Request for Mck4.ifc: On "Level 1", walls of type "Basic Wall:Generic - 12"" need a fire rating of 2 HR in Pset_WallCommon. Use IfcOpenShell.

First a look at what the model holds.

```python
import ifcopenshell
import ifcopenshell.util.element

model = ifcopenshell.open("Mck4.ifc")
print(model.schema)
storey = next(s for s in model.by_type("IfcBuildingStorey") if s.Name == "Level 1")
walls = [e for e in ifcopenshell.util.element.get_decomposition(storey) if e.is_a("IfcWall")]
seen = {}
for e in walls:
    element_type = ifcopenshell.util.element.get_type(e)
    key = (element_type.Name if element_type != e and element_type else None, ifcopenshell.util.element.get_pset(e, "Pset_WallCommon", "FireRating"))
    seen[key] = seen.get(key, 0) + 1
for (name, value), count in sorted(seen.items(), key=str):
    print(count, "x", name, "|", value)
```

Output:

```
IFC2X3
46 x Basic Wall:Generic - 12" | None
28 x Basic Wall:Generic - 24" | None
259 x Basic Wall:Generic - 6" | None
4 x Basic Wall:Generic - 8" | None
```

```python
import ifcopenshell
import ifcopenshell.api.pset
import ifcopenshell.util.element

model = ifcopenshell.open("Mck4.ifc")

storey = next(s for s in model.by_type("IfcBuildingStorey") if s.Name == "Level 1")
walls = [e for e in ifcopenshell.util.element.get_decomposition(storey) if e.is_a("IfcWall")]

count = 0
for e in walls:
    element_type = ifcopenshell.util.element.get_type(e)
    if element_type in (None, e) or element_type.Name != 'Basic Wall:Generic - 12"':
        continue
    # add_pset returns the element's existing set when there is one.
    pset = ifcopenshell.api.pset.add_pset(model, product=e, name="Pset_WallCommon")
    ifcopenshell.api.pset.edit_pset(model, pset=pset, properties={"FireRating": "2 HR"})
    count += 1

print(count, "walls updated")

model.write("Mck4_edited.ifc")
```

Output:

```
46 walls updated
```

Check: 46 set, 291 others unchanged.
